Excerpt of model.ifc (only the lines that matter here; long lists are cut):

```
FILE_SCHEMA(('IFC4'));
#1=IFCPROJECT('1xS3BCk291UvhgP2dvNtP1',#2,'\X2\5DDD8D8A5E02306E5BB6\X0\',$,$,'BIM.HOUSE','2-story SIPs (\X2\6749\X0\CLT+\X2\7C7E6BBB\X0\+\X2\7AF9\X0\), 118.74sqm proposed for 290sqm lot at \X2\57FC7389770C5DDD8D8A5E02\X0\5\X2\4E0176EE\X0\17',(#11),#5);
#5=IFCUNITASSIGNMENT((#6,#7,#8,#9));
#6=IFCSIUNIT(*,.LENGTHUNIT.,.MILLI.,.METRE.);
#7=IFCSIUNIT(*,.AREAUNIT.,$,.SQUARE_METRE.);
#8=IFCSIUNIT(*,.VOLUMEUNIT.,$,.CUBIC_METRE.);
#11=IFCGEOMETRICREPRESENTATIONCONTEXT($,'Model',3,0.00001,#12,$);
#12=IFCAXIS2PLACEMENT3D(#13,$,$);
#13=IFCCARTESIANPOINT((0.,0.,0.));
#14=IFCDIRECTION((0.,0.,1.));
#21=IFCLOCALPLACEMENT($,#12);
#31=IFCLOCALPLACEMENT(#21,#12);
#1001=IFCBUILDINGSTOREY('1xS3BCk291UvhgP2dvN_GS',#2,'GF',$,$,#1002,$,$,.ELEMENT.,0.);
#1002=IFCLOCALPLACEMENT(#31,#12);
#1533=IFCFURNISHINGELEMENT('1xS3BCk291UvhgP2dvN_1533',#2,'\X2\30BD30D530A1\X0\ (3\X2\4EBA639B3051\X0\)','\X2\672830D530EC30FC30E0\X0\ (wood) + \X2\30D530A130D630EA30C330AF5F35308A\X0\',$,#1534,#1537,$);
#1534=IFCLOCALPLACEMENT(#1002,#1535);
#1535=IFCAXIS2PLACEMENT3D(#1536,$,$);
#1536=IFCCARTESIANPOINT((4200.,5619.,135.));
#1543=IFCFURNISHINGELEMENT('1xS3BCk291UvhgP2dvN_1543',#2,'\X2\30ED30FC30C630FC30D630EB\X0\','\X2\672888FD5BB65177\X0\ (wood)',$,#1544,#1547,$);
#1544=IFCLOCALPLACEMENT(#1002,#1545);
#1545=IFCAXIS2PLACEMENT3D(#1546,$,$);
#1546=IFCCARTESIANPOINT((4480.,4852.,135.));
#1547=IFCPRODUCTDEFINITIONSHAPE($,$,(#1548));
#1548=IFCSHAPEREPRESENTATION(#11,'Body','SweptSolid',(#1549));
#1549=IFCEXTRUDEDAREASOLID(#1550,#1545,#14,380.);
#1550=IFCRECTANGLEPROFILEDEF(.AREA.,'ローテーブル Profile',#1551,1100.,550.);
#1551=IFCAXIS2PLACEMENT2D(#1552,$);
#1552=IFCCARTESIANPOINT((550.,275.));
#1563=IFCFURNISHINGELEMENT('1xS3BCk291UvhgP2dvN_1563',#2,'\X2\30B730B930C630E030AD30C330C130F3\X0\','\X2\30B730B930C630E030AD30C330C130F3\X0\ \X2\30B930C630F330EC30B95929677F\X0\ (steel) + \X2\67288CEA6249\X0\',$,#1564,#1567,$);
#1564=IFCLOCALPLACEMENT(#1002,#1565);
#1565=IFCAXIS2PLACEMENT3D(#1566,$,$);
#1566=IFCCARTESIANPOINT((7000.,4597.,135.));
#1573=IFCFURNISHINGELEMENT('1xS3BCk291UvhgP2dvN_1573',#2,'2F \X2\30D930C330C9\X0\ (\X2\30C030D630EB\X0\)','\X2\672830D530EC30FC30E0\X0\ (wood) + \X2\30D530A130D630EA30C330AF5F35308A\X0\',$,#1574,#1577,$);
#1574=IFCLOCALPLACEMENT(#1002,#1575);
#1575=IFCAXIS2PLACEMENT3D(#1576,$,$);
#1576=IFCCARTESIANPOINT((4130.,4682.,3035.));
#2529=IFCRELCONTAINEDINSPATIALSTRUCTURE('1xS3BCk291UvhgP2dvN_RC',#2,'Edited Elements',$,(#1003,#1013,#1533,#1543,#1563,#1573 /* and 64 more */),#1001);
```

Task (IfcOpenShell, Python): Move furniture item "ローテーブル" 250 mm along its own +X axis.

```python
import ifcopenshell
import ifcopenshell.api.geometry
import ifcopenshell.util.placement
import ifcopenshell.util.unit

model = ifcopenshell.open("model.ifc")
unit_scale = ifcopenshell.util.unit.calculate_unit_scale(model)

item = model.by_guid("1xS3BCk291UvhgP2dvN_1543")
matrix = ifcopenshell.util.placement.get_local_placement(item.ObjectPlacement)
matrix[:3, 3] += matrix[:3, 0] * 0.25 / unit_scale
ifcopenshell.api.geometry.edit_object_placement(model, product=item, matrix=matrix, is_si=False)

print(ifcopenshell.util.placement.get_local_placement(item.ObjectPlacement).round(3) + 0.0)

model.write("model_edited.ifc")
```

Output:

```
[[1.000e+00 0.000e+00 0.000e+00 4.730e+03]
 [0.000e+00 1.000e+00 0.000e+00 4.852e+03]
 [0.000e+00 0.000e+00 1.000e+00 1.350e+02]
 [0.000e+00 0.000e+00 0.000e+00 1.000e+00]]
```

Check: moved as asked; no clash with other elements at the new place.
